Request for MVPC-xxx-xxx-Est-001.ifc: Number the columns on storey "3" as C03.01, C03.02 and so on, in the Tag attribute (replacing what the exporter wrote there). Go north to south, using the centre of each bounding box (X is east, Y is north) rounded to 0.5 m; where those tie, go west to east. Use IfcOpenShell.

First a look at what the model holds.

```python
import ifcopenshell
import ifcopenshell.util.element
import ifcopenshell.util.placement

model = ifcopenshell.open("MVPC-xxx-xxx-Est-001.ifc")
print(model.schema)
storey = next(s for s in model.by_type("IfcBuildingStorey") if s.Name == "3")
columns = [e for e in ifcopenshell.util.element.get_decomposition(storey) if e.is_a("IfcColumn")]
for e in sorted(columns, key=lambda e: e.id()):
    origin = ifcopenshell.util.placement.get_local_placement(e.ObjectPlacement)[:3, 3]
    print(e.id(), e.Tag, e.Name, origin.round(2) + 0.0, sep=" | ")
```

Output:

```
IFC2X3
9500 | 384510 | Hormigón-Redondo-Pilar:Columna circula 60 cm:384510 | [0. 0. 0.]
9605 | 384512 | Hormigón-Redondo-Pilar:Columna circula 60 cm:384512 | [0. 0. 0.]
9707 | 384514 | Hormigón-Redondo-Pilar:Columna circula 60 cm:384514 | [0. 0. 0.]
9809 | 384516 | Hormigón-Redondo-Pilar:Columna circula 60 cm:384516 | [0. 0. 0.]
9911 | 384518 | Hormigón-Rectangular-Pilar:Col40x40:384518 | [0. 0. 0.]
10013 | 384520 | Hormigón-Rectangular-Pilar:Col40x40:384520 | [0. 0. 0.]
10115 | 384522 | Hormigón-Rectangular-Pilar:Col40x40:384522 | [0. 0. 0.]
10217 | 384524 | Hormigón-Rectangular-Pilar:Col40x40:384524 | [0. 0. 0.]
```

```python
import ifcopenshell
import ifcopenshell.geom
import ifcopenshell.util.element
import ifcopenshell.util.shape

model = ifcopenshell.open("MVPC-xxx-xxx-Est-001.ifc")
settings = ifcopenshell.geom.settings()
settings.set("use-world-coords", True)


def centre(element):
    shape = ifcopenshell.geom.create_shape(settings, element)
    return ifcopenshell.util.shape.get_bbox_centroid(shape.geometry)


storey = next(s for s in model.by_type("IfcBuildingStorey") if s.Name == "3")
columns = [e for e in ifcopenshell.util.element.get_decomposition(storey) if e.is_a("IfcColumn")]

# Insertion points can sit at a corner or the storey origin, so sort by the geometry (in metres).
centres = {e: centre(e) for e in columns}
columns.sort(key=lambda e: (-round(centres[e][1] / 0.5), centres[e][0]))

for i, e in enumerate(columns, start=1):
    number = f"C03.{i:02d}"
    e.Tag = number
    print(e.id(), number)

model.write("MVPC-xxx-xxx-Est-001_updated.ifc")
```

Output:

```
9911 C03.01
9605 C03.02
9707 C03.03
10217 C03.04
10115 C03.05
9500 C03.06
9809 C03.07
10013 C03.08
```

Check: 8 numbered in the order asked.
